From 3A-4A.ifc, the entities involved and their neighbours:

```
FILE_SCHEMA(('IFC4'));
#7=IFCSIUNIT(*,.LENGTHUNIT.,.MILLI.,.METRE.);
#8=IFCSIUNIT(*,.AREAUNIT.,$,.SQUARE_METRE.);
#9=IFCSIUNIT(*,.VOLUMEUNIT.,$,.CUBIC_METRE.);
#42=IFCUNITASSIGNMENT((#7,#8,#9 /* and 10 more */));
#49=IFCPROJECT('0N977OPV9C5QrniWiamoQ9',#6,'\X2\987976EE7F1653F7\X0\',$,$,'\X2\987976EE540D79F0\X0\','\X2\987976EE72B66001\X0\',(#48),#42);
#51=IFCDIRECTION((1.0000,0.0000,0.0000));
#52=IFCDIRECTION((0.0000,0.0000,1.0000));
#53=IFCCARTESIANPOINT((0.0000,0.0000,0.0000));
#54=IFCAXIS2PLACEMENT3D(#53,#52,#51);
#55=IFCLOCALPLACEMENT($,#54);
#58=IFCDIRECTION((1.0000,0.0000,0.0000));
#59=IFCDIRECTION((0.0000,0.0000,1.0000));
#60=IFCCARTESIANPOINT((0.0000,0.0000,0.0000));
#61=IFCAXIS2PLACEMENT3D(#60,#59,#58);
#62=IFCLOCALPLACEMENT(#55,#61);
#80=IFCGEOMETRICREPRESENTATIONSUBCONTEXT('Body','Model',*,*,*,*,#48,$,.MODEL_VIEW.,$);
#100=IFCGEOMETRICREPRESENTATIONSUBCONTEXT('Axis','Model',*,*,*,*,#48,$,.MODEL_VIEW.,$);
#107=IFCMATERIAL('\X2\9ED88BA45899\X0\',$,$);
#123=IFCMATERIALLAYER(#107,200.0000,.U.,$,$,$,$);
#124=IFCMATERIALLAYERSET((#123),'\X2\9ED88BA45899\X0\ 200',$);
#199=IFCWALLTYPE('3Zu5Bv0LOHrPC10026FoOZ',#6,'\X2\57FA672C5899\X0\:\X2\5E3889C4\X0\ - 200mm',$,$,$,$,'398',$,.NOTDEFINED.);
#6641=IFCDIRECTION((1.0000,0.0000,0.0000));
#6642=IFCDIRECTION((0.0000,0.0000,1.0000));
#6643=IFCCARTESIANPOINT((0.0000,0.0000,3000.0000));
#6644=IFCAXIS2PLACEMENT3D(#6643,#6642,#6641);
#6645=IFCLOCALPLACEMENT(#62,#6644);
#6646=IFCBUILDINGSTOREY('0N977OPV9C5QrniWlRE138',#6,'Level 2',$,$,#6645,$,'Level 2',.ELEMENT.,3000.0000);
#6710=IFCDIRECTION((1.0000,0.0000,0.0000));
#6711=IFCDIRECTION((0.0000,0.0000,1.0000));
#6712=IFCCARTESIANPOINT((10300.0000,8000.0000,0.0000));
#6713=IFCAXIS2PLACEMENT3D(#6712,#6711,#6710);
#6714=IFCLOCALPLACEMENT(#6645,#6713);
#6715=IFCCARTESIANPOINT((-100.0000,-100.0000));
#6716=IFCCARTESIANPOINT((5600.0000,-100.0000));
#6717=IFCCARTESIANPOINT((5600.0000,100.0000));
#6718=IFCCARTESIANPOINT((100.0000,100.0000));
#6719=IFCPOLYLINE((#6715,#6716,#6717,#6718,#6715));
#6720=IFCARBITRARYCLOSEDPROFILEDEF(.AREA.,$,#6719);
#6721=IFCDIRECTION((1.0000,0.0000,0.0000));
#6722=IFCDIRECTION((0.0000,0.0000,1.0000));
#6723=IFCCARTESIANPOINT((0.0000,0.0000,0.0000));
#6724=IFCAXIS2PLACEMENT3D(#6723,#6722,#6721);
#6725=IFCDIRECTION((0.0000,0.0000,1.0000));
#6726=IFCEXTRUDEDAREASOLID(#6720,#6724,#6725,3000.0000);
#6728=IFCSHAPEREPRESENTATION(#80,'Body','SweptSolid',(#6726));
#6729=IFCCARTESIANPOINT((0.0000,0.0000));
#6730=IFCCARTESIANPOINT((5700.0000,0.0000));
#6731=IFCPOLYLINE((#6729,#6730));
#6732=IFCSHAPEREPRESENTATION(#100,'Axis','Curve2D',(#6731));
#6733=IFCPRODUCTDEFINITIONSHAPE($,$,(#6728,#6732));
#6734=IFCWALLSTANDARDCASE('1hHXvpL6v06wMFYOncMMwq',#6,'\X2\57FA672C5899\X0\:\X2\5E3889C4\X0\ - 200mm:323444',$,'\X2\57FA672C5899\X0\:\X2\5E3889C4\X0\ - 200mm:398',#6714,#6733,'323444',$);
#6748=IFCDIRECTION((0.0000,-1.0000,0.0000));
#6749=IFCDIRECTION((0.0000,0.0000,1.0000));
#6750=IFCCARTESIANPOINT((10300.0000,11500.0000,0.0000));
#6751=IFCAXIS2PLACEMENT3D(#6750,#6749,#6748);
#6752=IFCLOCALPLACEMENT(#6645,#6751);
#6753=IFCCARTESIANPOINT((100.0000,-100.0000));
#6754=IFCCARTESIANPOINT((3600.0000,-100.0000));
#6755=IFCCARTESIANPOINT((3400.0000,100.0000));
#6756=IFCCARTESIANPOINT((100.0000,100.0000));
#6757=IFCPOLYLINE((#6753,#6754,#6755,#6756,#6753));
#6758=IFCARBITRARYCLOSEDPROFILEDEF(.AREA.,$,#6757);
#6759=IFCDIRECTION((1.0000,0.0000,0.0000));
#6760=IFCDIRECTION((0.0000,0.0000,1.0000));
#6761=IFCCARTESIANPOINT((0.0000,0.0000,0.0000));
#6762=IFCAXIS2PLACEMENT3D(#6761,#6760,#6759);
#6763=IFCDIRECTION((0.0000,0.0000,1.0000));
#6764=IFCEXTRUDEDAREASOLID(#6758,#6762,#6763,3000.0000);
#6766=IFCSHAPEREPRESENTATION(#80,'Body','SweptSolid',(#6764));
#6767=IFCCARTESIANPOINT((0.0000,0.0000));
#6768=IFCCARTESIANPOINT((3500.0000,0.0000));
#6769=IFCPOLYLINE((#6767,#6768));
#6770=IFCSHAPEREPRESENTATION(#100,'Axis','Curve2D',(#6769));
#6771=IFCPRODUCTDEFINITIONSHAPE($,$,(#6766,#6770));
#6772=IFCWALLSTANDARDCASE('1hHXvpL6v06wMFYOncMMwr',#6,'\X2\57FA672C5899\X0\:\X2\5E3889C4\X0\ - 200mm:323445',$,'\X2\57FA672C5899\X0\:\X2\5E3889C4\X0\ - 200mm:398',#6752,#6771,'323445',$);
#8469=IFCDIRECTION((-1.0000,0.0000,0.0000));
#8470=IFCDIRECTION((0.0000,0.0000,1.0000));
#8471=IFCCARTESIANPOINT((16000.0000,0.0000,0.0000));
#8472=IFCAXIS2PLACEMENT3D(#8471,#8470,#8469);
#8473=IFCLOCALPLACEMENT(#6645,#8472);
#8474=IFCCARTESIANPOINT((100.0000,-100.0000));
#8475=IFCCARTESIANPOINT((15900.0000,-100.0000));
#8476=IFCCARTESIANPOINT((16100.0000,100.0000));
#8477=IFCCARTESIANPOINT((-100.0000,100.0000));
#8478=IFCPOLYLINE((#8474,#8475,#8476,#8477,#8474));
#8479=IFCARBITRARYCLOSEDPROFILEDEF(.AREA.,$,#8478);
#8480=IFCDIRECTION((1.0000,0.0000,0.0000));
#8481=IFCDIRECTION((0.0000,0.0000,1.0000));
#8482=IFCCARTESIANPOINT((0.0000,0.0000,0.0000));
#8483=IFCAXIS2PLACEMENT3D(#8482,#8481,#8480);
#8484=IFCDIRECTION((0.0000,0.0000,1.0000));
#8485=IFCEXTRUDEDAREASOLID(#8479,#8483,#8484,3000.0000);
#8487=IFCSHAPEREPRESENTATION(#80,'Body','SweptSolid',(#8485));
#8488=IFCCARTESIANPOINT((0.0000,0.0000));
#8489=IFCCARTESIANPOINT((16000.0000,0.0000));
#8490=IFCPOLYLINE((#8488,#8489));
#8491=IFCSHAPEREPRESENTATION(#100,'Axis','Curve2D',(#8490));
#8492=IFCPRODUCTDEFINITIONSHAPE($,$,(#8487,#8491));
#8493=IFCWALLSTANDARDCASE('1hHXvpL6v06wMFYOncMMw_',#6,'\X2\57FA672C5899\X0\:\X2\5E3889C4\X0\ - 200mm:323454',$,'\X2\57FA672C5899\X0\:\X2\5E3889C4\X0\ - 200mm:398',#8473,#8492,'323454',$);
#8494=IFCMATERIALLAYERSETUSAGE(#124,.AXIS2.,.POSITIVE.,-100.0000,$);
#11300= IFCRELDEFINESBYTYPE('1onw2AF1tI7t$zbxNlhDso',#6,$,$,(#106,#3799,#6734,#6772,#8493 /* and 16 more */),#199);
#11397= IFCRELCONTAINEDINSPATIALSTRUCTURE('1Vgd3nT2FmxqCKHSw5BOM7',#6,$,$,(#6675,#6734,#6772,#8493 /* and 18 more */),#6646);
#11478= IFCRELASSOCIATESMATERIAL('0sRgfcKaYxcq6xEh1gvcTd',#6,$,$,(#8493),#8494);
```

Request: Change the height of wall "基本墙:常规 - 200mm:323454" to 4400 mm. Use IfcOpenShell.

```python
import ifcopenshell
import ifcopenshell.geom
import ifcopenshell.util.representation
import ifcopenshell.util.shape
import ifcopenshell.util.unit

model = ifcopenshell.open("3A-4A.ifc")
unit_scale = ifcopenshell.util.unit.calculate_unit_scale(model)
settings = ifcopenshell.geom.settings()


def volume(element):
    """Net volume in cubic metres, openings subtracted."""
    shape = ifcopenshell.geom.create_shape(settings, element)
    return ifcopenshell.util.shape.get_volume(shape.geometry)


wall = model.by_guid("1hHXvpL6v06wMFYOncMMw_")
before = volume(wall)

body = ifcopenshell.util.representation.get_representation(wall, "Model", "Body")
solid = body.Items[0]
old_height = solid.Depth
solid.Depth = 4.4 / unit_scale
after = volume(wall)

print(f"height {old_height:g} -> {solid.Depth:g}, volume {before:.3f} -> {after:.3f} m3")

model.write("3A-4A_rev.ifc")
```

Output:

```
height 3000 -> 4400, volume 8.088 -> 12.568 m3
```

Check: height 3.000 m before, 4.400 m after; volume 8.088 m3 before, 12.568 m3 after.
